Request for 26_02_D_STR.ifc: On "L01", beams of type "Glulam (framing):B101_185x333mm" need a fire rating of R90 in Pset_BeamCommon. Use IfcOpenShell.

First a look at what the model holds.

```python
import ifcopenshell
import ifcopenshell.util.element

model = ifcopenshell.open("26_02_D_STR.ifc")
print(model.schema)
storey = next(s for s in model.by_type("IfcBuildingStorey") if s.Name == "L01")
beams = [e for e in ifcopenshell.util.element.get_decomposition(storey) if e.is_a("IfcBeam")]
seen = {}
for e in beams:
    element_type = ifcopenshell.util.element.get_type(e)
    key = (element_type.Name if element_type != e and element_type else None, ifcopenshell.util.element.get_pset(e, "Pset_BeamCommon", "FireRating"))
    seen[key] = seen.get(key, 0) + 1
for (name, value), count in sorted(seen.items(), key=str):
    print(count, "x", name, "|", value)
```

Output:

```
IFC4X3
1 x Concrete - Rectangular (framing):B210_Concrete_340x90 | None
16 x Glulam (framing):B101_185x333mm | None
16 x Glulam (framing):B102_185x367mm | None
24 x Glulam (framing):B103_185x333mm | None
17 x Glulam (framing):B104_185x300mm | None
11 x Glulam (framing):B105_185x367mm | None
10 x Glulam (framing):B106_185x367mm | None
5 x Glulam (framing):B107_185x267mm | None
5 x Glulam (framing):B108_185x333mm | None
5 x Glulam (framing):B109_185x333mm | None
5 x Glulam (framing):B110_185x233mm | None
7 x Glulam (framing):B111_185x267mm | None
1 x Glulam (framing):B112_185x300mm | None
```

```python
import ifcopenshell
import ifcopenshell.api.pset
import ifcopenshell.util.element

model = ifcopenshell.open("26_02_D_STR.ifc")

storey = next(s for s in model.by_type("IfcBuildingStorey") if s.Name == "L01")
beams = [e for e in ifcopenshell.util.element.get_decomposition(storey) if e.is_a("IfcBeam")]

count = 0
for e in beams:
    element_type = ifcopenshell.util.element.get_type(e)
    if element_type in (None, e) or element_type.Name != "Glulam (framing):B101_185x333mm":
        continue
    # add_pset returns the element's existing set when there is one.
    pset = ifcopenshell.api.pset.add_pset(model, product=e, name="Pset_BeamCommon")
    ifcopenshell.api.pset.edit_pset(model, pset=pset, properties={"FireRating": "R90"})
    count += 1

print(count, "beams updated")

model.write("26_02_D_STR_v2.ifc")
```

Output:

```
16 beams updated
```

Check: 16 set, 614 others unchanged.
